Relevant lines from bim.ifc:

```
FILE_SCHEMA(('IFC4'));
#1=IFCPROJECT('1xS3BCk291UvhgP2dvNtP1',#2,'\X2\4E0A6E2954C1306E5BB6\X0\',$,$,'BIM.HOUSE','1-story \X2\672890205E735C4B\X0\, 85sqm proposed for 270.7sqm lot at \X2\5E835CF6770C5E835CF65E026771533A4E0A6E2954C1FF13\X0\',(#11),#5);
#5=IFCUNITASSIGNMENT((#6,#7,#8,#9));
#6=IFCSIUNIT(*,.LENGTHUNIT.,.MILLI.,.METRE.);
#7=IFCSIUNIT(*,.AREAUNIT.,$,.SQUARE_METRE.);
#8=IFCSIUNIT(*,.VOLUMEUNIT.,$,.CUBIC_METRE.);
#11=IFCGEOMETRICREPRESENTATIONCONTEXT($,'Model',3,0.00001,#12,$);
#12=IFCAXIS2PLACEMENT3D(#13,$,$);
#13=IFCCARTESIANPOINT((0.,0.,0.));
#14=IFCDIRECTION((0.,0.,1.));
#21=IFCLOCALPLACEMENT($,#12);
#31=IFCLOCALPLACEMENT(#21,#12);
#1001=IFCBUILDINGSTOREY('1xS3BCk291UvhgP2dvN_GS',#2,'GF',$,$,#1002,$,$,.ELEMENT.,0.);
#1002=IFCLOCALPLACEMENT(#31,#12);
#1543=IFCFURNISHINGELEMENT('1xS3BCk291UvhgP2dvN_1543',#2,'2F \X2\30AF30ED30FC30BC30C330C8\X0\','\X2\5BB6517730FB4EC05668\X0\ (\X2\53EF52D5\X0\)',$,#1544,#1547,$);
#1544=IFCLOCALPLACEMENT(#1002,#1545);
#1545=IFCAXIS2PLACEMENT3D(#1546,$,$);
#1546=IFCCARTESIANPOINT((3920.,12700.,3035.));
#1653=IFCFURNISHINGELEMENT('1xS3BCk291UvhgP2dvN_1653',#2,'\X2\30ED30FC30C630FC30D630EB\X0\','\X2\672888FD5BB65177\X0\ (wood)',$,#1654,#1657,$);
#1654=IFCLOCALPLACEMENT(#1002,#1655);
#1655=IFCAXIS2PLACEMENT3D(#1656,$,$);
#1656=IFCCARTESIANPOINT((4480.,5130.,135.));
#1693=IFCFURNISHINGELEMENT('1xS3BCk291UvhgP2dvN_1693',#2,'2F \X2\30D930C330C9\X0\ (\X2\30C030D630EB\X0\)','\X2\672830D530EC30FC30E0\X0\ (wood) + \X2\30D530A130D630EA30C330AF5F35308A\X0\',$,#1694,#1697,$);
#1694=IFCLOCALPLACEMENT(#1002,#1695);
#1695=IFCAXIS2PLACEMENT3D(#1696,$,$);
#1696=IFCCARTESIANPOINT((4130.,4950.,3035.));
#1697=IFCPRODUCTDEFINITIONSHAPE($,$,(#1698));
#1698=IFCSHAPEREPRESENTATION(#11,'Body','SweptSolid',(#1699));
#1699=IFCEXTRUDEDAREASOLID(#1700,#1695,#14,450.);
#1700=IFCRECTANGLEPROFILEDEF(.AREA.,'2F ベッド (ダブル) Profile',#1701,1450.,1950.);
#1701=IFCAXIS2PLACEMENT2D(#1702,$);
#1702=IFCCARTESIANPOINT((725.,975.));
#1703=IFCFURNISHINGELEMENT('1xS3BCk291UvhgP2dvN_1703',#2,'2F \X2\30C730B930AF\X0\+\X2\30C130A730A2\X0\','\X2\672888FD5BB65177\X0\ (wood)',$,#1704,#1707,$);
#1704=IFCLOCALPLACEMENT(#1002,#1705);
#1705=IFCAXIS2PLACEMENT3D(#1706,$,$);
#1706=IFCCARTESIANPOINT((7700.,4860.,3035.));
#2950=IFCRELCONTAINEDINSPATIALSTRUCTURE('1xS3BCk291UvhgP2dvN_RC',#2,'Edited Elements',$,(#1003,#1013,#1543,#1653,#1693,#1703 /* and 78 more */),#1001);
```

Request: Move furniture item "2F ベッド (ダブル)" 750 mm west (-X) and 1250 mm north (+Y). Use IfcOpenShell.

```python
import ifcopenshell
import ifcopenshell.api.geometry
import ifcopenshell.util.placement
import ifcopenshell.util.unit

model = ifcopenshell.open("bim.ifc")
unit_scale = ifcopenshell.util.unit.calculate_unit_scale(model)

item = model.by_guid("1xS3BCk291UvhgP2dvN_1693")
matrix = ifcopenshell.util.placement.get_local_placement(item.ObjectPlacement)
matrix[0, 3] -= 0.75 / unit_scale
matrix[1, 3] += 1.25 / unit_scale
ifcopenshell.api.geometry.edit_object_placement(model, product=item, matrix=matrix, is_si=False)

print(ifcopenshell.util.placement.get_local_placement(item.ObjectPlacement).round(3) + 0.0)

model.write("bim-out.ifc")
```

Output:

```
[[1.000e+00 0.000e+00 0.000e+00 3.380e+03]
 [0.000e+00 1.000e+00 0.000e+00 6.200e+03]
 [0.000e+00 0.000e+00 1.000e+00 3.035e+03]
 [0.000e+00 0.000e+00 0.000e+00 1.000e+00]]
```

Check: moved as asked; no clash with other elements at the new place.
